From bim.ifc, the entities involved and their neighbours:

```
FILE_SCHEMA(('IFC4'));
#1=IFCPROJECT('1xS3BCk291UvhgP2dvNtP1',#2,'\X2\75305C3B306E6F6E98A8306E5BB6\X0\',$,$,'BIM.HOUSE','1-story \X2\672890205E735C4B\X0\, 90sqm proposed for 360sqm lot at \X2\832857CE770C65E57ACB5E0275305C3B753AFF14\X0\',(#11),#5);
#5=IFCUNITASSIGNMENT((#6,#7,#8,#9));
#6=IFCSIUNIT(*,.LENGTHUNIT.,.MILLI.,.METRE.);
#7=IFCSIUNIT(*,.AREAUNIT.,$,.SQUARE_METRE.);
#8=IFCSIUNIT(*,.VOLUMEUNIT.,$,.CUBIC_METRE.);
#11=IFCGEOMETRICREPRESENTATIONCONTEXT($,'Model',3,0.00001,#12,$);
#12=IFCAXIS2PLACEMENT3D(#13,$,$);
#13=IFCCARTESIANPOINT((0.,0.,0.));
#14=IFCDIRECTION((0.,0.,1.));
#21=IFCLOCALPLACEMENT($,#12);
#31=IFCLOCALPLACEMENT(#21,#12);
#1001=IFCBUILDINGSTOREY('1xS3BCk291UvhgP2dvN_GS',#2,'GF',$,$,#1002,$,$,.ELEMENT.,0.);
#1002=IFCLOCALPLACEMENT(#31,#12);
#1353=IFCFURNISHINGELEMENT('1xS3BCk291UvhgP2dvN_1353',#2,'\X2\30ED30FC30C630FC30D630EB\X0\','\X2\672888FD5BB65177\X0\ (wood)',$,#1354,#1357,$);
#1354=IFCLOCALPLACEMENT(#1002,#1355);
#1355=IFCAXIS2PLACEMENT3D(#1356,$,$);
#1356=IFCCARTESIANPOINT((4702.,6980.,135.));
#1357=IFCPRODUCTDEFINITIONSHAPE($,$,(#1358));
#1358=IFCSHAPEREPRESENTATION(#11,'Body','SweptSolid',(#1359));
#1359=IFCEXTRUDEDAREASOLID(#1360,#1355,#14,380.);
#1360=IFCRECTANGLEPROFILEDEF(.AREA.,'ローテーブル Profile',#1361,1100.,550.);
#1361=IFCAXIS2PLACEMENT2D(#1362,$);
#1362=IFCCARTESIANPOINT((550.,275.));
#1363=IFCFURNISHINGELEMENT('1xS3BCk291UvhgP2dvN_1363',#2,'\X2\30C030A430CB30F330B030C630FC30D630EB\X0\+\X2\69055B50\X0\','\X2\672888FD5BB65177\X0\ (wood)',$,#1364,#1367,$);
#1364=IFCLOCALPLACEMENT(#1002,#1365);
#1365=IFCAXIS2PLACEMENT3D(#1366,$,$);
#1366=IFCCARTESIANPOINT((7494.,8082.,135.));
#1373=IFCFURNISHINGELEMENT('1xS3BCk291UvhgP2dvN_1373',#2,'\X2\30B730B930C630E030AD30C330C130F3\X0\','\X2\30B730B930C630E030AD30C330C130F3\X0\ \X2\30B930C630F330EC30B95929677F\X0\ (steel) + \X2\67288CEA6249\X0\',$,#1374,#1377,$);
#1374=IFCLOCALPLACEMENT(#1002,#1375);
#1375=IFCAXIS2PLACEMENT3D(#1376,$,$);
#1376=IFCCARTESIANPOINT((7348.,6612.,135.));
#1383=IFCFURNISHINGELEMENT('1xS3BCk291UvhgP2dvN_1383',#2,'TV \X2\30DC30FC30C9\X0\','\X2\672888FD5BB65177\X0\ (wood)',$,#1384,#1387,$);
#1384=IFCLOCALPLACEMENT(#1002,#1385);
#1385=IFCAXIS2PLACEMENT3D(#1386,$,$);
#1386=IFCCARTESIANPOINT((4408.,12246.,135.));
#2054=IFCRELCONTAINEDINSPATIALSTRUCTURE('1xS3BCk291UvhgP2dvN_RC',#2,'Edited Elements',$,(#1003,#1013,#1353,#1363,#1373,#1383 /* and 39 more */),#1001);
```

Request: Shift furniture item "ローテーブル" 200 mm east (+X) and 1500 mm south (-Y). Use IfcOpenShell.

```python
import ifcopenshell
import ifcopenshell.api.geometry
import ifcopenshell.util.placement
import ifcopenshell.util.unit

model = ifcopenshell.open("bim.ifc")
unit_scale = ifcopenshell.util.unit.calculate_unit_scale(model)

item = model.by_id(1353)
matrix = ifcopenshell.util.placement.get_local_placement(item.ObjectPlacement)
matrix[0, 3] += 0.2 / unit_scale
matrix[1, 3] -= 1.5 / unit_scale
ifcopenshell.api.geometry.edit_object_placement(model, product=item, matrix=matrix, is_si=False)

print(ifcopenshell.util.placement.get_local_placement(item.ObjectPlacement).round(3) + 0.0)

model.write("bim_v2.ifc")
```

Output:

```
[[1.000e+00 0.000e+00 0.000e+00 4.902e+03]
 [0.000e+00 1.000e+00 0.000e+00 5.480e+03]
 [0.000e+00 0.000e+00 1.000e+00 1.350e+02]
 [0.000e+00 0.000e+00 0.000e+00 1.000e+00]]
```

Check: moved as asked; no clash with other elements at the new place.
